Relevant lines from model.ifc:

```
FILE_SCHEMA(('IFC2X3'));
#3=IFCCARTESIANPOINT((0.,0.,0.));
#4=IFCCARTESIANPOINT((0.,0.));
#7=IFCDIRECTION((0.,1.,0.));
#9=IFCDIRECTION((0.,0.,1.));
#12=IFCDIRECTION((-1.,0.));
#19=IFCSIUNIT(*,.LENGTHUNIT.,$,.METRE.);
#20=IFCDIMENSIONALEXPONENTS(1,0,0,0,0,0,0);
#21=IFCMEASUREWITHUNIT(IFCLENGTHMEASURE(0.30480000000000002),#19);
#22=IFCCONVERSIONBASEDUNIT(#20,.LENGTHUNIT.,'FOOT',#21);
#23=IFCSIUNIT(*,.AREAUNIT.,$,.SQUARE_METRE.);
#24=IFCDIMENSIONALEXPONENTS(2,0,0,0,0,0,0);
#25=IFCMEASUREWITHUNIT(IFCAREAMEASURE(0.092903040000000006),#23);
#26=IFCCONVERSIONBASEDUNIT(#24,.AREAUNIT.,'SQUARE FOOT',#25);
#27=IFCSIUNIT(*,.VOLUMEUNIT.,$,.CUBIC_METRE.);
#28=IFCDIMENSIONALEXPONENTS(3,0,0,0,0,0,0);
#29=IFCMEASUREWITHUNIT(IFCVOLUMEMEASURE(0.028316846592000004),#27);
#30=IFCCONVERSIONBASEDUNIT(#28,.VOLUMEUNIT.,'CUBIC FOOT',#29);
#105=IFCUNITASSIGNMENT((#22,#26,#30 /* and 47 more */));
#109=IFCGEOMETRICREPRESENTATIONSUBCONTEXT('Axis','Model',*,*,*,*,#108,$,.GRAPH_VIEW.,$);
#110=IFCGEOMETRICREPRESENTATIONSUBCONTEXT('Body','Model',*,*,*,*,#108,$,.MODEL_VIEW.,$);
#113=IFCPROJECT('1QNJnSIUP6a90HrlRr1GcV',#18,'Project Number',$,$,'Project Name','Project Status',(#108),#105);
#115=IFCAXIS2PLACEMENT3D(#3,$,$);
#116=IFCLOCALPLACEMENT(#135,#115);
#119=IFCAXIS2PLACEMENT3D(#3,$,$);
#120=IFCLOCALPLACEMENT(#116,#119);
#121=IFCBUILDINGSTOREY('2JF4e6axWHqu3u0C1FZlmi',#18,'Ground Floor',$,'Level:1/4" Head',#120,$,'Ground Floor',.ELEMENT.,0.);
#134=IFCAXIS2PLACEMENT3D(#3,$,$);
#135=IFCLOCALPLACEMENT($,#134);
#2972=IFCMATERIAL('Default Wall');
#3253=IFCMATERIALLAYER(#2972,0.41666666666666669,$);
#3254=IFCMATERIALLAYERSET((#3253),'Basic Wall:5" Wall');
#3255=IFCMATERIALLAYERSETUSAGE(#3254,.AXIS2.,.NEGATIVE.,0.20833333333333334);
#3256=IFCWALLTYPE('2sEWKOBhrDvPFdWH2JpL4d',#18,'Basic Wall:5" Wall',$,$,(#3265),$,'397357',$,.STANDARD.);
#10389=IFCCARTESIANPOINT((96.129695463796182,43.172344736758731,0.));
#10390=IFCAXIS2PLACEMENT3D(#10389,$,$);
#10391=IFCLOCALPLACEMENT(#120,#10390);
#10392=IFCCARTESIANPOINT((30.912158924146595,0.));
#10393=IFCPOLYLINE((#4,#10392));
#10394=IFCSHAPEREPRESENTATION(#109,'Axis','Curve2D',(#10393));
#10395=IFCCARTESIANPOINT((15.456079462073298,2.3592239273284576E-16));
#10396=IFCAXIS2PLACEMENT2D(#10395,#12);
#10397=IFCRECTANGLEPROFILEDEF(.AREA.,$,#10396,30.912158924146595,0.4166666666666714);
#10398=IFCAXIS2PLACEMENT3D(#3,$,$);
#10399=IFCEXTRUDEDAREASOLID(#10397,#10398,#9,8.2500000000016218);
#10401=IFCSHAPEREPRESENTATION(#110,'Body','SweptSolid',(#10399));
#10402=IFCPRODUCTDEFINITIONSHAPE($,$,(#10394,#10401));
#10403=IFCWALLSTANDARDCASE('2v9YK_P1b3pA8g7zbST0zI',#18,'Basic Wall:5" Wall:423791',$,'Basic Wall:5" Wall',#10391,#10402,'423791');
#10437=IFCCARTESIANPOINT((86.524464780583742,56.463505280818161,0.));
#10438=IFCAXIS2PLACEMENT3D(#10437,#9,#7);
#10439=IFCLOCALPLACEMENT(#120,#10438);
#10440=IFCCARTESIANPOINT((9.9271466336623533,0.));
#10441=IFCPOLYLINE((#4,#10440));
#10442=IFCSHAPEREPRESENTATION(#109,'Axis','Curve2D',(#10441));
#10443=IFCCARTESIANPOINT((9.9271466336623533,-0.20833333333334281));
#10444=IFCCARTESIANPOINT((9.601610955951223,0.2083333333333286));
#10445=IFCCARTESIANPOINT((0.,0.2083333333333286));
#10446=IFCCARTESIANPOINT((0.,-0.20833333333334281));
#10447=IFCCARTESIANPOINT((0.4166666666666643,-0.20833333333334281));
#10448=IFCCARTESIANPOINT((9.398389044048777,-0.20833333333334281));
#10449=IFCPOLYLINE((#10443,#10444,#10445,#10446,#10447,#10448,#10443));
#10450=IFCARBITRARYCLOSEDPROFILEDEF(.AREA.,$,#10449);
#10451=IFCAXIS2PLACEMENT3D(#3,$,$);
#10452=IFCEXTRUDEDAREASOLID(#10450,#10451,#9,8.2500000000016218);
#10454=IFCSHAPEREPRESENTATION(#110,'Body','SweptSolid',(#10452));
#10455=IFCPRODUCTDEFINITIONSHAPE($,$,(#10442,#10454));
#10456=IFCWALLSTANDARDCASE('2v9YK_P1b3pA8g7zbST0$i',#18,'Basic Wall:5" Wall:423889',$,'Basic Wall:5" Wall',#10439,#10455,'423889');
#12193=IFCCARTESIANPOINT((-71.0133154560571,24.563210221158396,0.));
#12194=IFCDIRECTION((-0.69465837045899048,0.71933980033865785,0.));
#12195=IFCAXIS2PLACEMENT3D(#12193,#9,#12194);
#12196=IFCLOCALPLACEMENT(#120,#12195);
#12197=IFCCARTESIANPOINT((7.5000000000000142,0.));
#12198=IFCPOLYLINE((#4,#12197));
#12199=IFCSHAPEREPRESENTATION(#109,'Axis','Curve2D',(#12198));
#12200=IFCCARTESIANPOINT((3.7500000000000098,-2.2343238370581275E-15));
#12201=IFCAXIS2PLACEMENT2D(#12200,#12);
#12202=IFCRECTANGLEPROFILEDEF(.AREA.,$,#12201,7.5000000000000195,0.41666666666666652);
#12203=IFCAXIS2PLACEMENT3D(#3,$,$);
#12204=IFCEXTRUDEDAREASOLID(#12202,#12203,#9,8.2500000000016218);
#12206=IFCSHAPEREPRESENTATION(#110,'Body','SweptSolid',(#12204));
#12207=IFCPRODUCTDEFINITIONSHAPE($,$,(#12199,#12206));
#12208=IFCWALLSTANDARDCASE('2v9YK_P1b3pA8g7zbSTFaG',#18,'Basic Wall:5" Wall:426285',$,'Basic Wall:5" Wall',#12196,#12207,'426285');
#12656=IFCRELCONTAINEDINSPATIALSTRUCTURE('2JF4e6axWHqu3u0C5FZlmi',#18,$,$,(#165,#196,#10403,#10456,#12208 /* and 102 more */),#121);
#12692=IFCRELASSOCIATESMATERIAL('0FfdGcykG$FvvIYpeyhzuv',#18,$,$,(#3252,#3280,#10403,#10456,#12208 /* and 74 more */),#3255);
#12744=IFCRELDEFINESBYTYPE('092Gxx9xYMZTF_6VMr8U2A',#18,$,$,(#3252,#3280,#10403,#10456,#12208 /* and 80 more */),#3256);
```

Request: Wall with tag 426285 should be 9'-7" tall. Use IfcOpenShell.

```python
import ifcopenshell
import ifcopenshell.geom
import ifcopenshell.util.representation
import ifcopenshell.util.shape
import ifcopenshell.util.unit

model = ifcopenshell.open("model.ifc")
unit_scale = ifcopenshell.util.unit.calculate_unit_scale(model)
settings = ifcopenshell.geom.settings()


def volume(element):
    """Net volume in cubic metres, openings subtracted."""
    shape = ifcopenshell.geom.create_shape(settings, element)
    return ifcopenshell.util.shape.get_volume(shape.geometry)


wall = model.by_guid("2v9YK_P1b3pA8g7zbSTFaG")
before = volume(wall)

body = ifcopenshell.util.representation.get_representation(wall, "Model", "Body")
solid = body.Items[0]
old_height = solid.Depth
solid.Depth = 115 * 0.0254 / unit_scale
after = volume(wall)

print(f"height {old_height:g} -> {solid.Depth:g}, volume {before:.3f} -> {after:.3f} m3")

model.write("model_updated.ifc")
```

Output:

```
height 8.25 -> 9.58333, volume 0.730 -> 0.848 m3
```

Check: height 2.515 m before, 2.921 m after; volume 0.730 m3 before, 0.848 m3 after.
